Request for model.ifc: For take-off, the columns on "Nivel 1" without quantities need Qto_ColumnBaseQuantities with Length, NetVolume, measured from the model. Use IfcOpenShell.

First a look at what the model holds.

```python
import ifcopenshell
import ifcopenshell.util.element
import ifcopenshell.util.unit

model = ifcopenshell.open("model.ifc")
print(model.schema)
for unit_type in ("LENGTHUNIT", "AREAUNIT", "VOLUMEUNIT"):
    print(unit_type, ifcopenshell.util.unit.calculate_unit_scale(model, unit_type))
storey = next(s for s in model.by_type("IfcBuildingStorey") if s.Name == "Nivel 1")
columns = [e for e in ifcopenshell.util.element.get_decomposition(storey) if e.is_a("IfcColumn")]
for e in sorted(columns, key=lambda e: e.id()):
    print(e.id(), e.is_a(), e.Name, list(ifcopenshell.util.element.get_psets(e, qtos_only=True)), sep=" | ")
```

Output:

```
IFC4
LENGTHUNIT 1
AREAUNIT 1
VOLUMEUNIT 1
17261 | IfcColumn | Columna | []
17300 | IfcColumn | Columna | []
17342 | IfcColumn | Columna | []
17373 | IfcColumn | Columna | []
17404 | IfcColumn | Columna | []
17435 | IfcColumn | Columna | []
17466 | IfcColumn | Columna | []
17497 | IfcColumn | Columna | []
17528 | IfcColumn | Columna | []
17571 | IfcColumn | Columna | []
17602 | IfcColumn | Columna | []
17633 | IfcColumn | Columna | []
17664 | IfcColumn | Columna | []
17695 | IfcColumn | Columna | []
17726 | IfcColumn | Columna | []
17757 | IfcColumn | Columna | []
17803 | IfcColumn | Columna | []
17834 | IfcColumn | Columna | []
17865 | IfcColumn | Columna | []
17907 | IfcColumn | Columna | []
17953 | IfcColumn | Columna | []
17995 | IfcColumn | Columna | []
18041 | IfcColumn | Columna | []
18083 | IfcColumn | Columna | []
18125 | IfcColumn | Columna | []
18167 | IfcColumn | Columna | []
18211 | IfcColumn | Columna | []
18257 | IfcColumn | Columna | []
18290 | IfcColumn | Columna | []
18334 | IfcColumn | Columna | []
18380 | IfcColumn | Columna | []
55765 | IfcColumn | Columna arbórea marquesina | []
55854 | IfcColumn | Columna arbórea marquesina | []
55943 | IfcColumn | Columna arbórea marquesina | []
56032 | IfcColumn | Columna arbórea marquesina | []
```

```python
import ifcopenshell
import ifcopenshell.api.pset
import ifcopenshell.geom
import ifcopenshell.util.element
import ifcopenshell.util.shape
import ifcopenshell.util.unit

model = ifcopenshell.open("model.ifc")
unit_scale = ifcopenshell.util.unit.calculate_unit_scale(model)
volume_scale = ifcopenshell.util.unit.calculate_unit_scale(model, "VOLUMEUNIT")
settings = ifcopenshell.geom.settings()

storey = next(s for s in model.by_type("IfcBuildingStorey") if s.Name == "Nivel 1")
columns = [e for e in ifcopenshell.util.element.get_decomposition(storey) if e.is_a("IfcColumn")]

for e in sorted(columns, key=lambda e: e.id()):
    if ifcopenshell.util.element.get_psets(e, qtos_only=True, should_inherit=False):
        continue
    # Geometry comes back in metres, in the element's own axes.
    shape = ifcopenshell.geom.create_shape(settings, e)
    values = {
        "Length": ifcopenshell.util.shape.get_z(shape.geometry) / unit_scale,
        "NetVolume": ifcopenshell.util.shape.get_volume(shape.geometry) / volume_scale,
    }
    qto = ifcopenshell.api.pset.add_qto(model, product=e, name="Qto_ColumnBaseQuantities")
    ifcopenshell.api.pset.edit_qto(model, qto=qto, properties=values)
    print(e.id(), {k: round(v, 3) for k, v in values.items()})

model.write("model_v2.ifc")
```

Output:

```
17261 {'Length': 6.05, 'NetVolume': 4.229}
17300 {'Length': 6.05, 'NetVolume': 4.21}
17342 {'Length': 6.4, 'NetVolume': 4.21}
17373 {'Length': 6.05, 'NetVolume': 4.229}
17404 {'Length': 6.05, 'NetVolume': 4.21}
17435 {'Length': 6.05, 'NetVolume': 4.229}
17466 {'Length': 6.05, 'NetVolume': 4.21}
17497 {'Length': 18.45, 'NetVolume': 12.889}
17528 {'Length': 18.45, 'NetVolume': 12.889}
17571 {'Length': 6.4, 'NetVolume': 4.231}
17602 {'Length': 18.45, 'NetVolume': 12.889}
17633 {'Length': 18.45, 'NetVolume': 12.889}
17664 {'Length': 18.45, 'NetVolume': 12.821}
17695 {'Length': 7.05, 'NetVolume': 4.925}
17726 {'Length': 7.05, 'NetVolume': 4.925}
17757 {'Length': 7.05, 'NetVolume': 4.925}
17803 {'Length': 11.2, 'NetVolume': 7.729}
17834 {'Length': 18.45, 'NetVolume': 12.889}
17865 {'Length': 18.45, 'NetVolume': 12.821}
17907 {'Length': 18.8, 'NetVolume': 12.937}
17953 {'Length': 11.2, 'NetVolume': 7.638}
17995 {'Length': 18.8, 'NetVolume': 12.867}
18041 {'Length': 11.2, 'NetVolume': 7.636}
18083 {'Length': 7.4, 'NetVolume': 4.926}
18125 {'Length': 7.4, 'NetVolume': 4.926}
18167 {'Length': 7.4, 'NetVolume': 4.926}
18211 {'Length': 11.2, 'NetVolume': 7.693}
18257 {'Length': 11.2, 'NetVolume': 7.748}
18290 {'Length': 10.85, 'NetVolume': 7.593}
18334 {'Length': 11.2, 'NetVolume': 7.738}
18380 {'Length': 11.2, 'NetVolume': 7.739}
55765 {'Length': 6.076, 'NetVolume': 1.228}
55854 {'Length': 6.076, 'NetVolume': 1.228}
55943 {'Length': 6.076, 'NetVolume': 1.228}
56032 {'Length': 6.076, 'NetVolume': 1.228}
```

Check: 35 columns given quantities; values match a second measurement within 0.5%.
